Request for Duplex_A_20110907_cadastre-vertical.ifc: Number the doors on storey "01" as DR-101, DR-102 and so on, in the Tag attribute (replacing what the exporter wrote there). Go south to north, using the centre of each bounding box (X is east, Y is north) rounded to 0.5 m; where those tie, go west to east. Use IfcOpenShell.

First a look at what the model holds.

```python
import ifcopenshell
import ifcopenshell.util.element
import ifcopenshell.util.placement

model = ifcopenshell.open("Duplex_A_20110907_cadastre-vertical.ifc")
print(model.schema)
storey = next(s for s in model.by_type("IfcBuildingStorey") if s.Name == "01")
doors = [e for e in ifcopenshell.util.element.get_decomposition(storey) if e.is_a("IfcDoor")]
for e in sorted(doors, key=lambda e: e.id()):
    origin = ifcopenshell.util.placement.get_local_placement(e.ObjectPlacement)[:3, 3]
    print(e.id(), e.Tag, e.Name, origin.round(2) + 0.0, sep=" | ")
```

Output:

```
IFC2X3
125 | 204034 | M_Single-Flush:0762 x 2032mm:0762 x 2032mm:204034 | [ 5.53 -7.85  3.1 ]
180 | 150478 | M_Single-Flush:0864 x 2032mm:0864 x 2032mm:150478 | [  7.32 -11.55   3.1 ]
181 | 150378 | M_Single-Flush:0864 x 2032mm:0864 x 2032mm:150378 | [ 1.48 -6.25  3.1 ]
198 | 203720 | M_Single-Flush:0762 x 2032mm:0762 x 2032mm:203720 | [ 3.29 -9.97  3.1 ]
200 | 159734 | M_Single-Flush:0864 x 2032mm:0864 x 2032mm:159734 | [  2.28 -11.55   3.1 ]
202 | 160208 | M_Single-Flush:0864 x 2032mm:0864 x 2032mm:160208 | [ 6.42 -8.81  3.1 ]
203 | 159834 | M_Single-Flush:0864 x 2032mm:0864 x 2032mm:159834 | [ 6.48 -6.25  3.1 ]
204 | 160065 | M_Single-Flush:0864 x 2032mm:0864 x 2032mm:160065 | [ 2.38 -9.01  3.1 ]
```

```python
import ifcopenshell
import ifcopenshell.geom
import ifcopenshell.util.element
import ifcopenshell.util.shape

model = ifcopenshell.open("Duplex_A_20110907_cadastre-vertical.ifc")
settings = ifcopenshell.geom.settings()
settings.set("use-world-coords", True)


def centre(element):
    shape = ifcopenshell.geom.create_shape(settings, element)
    return ifcopenshell.util.shape.get_bbox_centroid(shape.geometry)


storey = next(s for s in model.by_type("IfcBuildingStorey") if s.Name == "01")
doors = [e for e in ifcopenshell.util.element.get_decomposition(storey) if e.is_a("IfcDoor")]

# Insertion points can sit at a corner or the storey origin, so sort by the geometry (in metres).
centres = {e: centre(e) for e in doors}
doors.sort(key=lambda e: (round(centres[e][1] / 0.5), centres[e][0]))

for i, e in enumerate(doors, start=1):
    number = f"DR-1{i:02d}"
    e.Tag = number
    print(e.id(), number)

model.write("Duplex_A_20110907_cadastre-vertical_v2.ifc")
```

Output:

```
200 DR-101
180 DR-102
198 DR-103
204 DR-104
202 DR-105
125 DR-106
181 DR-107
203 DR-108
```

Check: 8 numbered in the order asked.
